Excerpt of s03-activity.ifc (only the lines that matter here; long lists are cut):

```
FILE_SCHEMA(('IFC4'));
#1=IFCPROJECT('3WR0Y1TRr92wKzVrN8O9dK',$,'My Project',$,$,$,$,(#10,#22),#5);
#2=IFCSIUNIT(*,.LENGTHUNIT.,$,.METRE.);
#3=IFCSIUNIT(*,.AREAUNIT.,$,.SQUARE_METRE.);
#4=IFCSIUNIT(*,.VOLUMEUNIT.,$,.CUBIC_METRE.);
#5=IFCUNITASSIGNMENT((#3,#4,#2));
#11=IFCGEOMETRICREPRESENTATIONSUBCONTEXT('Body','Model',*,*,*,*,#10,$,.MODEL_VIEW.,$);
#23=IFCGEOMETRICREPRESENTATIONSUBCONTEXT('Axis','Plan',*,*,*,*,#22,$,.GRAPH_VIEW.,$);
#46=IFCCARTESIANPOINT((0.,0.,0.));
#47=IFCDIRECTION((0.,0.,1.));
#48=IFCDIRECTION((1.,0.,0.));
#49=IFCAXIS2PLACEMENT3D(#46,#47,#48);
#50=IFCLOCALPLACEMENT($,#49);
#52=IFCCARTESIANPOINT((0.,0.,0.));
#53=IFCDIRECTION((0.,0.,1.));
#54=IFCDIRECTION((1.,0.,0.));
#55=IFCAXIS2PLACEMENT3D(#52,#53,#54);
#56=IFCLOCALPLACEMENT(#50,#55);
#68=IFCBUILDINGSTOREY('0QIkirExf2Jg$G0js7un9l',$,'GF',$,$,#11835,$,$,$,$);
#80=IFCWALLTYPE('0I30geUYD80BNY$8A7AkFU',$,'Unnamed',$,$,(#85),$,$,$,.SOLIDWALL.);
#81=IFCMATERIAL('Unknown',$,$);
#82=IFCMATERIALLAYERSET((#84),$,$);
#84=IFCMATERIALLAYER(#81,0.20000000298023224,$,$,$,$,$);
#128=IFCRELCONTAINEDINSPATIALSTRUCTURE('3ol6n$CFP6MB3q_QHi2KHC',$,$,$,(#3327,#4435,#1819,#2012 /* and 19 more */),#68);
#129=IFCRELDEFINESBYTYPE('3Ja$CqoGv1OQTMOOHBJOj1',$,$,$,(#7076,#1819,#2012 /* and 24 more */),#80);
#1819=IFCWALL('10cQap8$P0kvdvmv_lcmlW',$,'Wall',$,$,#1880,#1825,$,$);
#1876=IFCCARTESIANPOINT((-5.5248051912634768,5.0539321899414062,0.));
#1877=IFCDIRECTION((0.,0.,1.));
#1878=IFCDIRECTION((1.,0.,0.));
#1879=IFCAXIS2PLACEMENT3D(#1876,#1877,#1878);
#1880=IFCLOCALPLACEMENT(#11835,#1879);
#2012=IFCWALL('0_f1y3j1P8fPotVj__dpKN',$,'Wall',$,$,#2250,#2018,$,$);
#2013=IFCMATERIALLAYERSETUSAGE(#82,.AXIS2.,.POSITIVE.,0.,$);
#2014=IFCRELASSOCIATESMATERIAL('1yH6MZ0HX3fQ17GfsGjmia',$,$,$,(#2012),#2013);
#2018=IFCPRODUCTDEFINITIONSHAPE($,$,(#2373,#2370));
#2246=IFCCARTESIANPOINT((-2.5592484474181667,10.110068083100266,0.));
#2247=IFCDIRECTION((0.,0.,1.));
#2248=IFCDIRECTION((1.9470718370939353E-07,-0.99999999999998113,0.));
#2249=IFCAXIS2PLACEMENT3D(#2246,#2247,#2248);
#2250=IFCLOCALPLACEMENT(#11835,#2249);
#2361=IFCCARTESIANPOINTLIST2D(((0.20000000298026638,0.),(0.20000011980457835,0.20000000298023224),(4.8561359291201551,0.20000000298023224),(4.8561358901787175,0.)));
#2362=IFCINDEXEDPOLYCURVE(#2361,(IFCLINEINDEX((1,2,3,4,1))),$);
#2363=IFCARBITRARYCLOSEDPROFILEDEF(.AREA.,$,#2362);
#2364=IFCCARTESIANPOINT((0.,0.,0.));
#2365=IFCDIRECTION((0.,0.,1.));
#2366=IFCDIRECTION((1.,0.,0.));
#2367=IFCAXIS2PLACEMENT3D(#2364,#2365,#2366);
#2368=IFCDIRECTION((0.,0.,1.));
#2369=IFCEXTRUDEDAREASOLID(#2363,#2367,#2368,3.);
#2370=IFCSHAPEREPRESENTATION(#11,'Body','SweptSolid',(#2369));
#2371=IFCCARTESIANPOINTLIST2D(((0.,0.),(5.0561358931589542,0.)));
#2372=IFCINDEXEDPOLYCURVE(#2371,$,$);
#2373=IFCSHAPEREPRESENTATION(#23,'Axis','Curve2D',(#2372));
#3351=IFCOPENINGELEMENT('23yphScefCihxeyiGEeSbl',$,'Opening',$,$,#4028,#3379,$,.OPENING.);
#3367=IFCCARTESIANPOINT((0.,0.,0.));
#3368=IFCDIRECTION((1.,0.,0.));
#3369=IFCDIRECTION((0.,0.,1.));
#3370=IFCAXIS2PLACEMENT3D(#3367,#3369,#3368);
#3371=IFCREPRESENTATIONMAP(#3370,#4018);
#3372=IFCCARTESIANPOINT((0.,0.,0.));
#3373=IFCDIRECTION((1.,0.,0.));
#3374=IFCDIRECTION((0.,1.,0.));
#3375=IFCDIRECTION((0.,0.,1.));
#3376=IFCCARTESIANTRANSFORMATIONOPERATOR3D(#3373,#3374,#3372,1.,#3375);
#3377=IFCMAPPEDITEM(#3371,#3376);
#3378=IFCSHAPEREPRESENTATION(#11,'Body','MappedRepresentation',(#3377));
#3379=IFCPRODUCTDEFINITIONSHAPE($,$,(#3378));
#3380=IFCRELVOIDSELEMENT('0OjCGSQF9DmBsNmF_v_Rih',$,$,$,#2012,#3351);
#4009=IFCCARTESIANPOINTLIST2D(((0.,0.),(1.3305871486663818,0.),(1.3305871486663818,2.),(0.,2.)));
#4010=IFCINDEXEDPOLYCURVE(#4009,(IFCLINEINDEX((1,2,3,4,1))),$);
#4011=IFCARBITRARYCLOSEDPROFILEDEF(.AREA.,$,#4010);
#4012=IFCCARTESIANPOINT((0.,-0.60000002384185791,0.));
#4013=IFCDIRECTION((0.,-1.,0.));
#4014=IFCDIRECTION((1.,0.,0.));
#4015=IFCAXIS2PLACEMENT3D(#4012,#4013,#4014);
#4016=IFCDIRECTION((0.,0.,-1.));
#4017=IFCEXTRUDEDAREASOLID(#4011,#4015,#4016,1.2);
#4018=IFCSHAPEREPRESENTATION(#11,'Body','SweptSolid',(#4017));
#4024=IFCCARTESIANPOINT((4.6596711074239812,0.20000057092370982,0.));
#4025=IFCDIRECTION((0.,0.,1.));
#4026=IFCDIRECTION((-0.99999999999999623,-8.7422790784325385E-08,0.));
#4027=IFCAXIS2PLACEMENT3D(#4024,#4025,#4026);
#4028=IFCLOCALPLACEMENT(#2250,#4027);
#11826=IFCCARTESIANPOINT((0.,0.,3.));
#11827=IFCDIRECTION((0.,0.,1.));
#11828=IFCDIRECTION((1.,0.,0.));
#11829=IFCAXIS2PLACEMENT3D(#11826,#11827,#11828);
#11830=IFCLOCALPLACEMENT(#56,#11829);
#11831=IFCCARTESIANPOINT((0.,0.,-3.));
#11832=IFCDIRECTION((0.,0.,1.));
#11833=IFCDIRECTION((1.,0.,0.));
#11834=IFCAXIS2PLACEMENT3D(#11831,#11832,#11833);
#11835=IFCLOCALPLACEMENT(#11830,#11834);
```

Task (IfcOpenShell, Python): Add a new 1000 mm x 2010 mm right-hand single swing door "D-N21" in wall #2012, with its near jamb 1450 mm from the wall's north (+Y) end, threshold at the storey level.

```python
import numpy as np
import ifcopenshell
import ifcopenshell.api.feature
import ifcopenshell.api.geometry
import ifcopenshell.api.root
import ifcopenshell.api.spatial
import ifcopenshell.geom
import ifcopenshell.util.element
import ifcopenshell.util.placement
import ifcopenshell.util.representation
import ifcopenshell.util.shape
import ifcopenshell.util.unit

model = ifcopenshell.open("s03-activity.ifc")
unit_scale = ifcopenshell.util.unit.calculate_unit_scale(model)
settings = ifcopenshell.geom.settings()


def volume(element):
    """Net volume in cubic metres, openings subtracted."""
    shape = ifcopenshell.geom.create_shape(settings, element)
    return ifcopenshell.util.shape.get_volume(shape.geometry)


wall = model.by_id(2012)
storey = ifcopenshell.util.element.get_container(wall, ifc_class="IfcBuildingStorey")
context = ifcopenshell.util.representation.get_context(model, "Model", "Body", "MODEL_VIEW")
before = volume(wall)

width, height, from_end, sill = 1, 2.01, 1.45, 0.0  # metres

# The wall runs along its own X axis, and the end named is its -X end.
wall_shape = ifcopenshell.geom.create_shape(settings, wall)
x, y, z = ifcopenshell.util.shape.get_vertices(wall_shape.geometry).T
start = x.min() + from_end
face, thickness = float(y.min()), float(y.max() - y.min())
wall_matrix = ifcopenshell.util.placement.get_local_placement(wall.ObjectPlacement)
level = ifcopenshell.util.placement.get_local_placement(storey.ObjectPlacement)[2, 3]


def in_wall(x, y):
    """Placement at x, y metres in the wall's axes, at sill height."""
    matrix = wall_matrix.copy()
    matrix[:, 3] = wall_matrix @ np.array([x / unit_scale, y / unit_scale, 0.0, 1.0])
    matrix[2, 3] = level + sill / unit_scale
    return matrix


# Opening: a box that overshoots both wall faces by 50 mm.
opening = ifcopenshell.api.root.create_entity(model, ifc_class="IfcOpeningElement", predefined_type="OPENING")
box = ifcopenshell.api.geometry.add_wall_representation(
    model, context=context, length=width, height=height, thickness=thickness + 0.1
)
ifcopenshell.api.geometry.assign_representation(model, product=opening, representation=box)
ifcopenshell.api.geometry.edit_object_placement(model, product=opening, matrix=in_wall(start, face - 0.05), is_si=False)
ifcopenshell.api.feature.add_feature(model, feature=opening, element=wall)

door = ifcopenshell.api.root.create_entity(model, ifc_class="IfcDoor", name="D-N21", predefined_type="DOOR")
door.OverallWidth, door.OverallHeight = width / unit_scale, height / unit_scale
door.OperationType = "SINGLE_SWING_RIGHT"
body = ifcopenshell.api.geometry.add_door_representation(
    model,
    context=context,
    overall_width=door.OverallWidth,
    overall_height=door.OverallHeight,
    operation_type="SINGLE_SWING_RIGHT",
    lining_properties={"LiningDepth": thickness / unit_scale, "ThresholdDepth": thickness / unit_scale},
)
ifcopenshell.api.geometry.assign_representation(model, product=door, representation=body)
ifcopenshell.api.spatial.assign_container(model, products=[door], relating_structure=storey)
ifcopenshell.api.feature.add_filling(model, opening=opening, element=door)

# The lining spans the wall, so the door starts at the wall face.
ifcopenshell.api.geometry.edit_object_placement(model, product=door, matrix=in_wall(start, face), is_si=False)

after = volume(wall)

print(f"wall volume {before:.3f} -> {after:.3f} m3")

model.write("s03-activity_v2.ifc")
```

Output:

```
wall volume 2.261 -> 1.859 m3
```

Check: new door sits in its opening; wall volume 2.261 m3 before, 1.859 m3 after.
